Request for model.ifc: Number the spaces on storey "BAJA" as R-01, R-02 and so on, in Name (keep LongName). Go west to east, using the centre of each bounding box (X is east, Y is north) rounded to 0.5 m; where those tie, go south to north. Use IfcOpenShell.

First a look at what the model holds.

```python
import ifcopenshell
import ifcopenshell.util.element
import ifcopenshell.util.placement

model = ifcopenshell.open("model.ifc")
print(model.schema)
storey = next(s for s in model.by_type("IfcBuildingStorey") if s.Name == "BAJA")
spaces = [e for e in ifcopenshell.util.element.get_decomposition(storey) if e.is_a("IfcSpace")]
for e in sorted(spaces, key=lambda e: e.id()):
    origin = ifcopenshell.util.placement.get_local_placement(e.ObjectPlacement)[:3, 3]
    print(e.id(), e.Name, e.LongName, origin.round(2) + 0.0, sep=" | ")
```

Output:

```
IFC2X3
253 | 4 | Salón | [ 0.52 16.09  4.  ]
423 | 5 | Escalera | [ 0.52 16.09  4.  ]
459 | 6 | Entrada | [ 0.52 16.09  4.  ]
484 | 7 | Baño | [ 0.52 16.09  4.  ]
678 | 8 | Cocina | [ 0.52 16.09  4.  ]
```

```python
import ifcopenshell
import ifcopenshell.geom
import ifcopenshell.util.element
import ifcopenshell.util.shape

model = ifcopenshell.open("model.ifc")
settings = ifcopenshell.geom.settings()
settings.set("use-world-coords", True)


def centre(element):
    shape = ifcopenshell.geom.create_shape(settings, element)
    return ifcopenshell.util.shape.get_bbox_centroid(shape.geometry)


storey = next(s for s in model.by_type("IfcBuildingStorey") if s.Name == "BAJA")
spaces = [e for e in ifcopenshell.util.element.get_decomposition(storey) if e.is_a("IfcSpace")]

# Insertion points can sit at a corner or the storey origin, so sort by the geometry (in metres).
centres = {e: centre(e) for e in spaces}
spaces.sort(key=lambda e: (round(centres[e][0] / 0.5), centres[e][1]))

for i, e in enumerate(spaces, start=1):
    number = f"R-{i:02d}"
    e.Name = number
    print(e.id(), number)

model.write("model_updated.ifc")
```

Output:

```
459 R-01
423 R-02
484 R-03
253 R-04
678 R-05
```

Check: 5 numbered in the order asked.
